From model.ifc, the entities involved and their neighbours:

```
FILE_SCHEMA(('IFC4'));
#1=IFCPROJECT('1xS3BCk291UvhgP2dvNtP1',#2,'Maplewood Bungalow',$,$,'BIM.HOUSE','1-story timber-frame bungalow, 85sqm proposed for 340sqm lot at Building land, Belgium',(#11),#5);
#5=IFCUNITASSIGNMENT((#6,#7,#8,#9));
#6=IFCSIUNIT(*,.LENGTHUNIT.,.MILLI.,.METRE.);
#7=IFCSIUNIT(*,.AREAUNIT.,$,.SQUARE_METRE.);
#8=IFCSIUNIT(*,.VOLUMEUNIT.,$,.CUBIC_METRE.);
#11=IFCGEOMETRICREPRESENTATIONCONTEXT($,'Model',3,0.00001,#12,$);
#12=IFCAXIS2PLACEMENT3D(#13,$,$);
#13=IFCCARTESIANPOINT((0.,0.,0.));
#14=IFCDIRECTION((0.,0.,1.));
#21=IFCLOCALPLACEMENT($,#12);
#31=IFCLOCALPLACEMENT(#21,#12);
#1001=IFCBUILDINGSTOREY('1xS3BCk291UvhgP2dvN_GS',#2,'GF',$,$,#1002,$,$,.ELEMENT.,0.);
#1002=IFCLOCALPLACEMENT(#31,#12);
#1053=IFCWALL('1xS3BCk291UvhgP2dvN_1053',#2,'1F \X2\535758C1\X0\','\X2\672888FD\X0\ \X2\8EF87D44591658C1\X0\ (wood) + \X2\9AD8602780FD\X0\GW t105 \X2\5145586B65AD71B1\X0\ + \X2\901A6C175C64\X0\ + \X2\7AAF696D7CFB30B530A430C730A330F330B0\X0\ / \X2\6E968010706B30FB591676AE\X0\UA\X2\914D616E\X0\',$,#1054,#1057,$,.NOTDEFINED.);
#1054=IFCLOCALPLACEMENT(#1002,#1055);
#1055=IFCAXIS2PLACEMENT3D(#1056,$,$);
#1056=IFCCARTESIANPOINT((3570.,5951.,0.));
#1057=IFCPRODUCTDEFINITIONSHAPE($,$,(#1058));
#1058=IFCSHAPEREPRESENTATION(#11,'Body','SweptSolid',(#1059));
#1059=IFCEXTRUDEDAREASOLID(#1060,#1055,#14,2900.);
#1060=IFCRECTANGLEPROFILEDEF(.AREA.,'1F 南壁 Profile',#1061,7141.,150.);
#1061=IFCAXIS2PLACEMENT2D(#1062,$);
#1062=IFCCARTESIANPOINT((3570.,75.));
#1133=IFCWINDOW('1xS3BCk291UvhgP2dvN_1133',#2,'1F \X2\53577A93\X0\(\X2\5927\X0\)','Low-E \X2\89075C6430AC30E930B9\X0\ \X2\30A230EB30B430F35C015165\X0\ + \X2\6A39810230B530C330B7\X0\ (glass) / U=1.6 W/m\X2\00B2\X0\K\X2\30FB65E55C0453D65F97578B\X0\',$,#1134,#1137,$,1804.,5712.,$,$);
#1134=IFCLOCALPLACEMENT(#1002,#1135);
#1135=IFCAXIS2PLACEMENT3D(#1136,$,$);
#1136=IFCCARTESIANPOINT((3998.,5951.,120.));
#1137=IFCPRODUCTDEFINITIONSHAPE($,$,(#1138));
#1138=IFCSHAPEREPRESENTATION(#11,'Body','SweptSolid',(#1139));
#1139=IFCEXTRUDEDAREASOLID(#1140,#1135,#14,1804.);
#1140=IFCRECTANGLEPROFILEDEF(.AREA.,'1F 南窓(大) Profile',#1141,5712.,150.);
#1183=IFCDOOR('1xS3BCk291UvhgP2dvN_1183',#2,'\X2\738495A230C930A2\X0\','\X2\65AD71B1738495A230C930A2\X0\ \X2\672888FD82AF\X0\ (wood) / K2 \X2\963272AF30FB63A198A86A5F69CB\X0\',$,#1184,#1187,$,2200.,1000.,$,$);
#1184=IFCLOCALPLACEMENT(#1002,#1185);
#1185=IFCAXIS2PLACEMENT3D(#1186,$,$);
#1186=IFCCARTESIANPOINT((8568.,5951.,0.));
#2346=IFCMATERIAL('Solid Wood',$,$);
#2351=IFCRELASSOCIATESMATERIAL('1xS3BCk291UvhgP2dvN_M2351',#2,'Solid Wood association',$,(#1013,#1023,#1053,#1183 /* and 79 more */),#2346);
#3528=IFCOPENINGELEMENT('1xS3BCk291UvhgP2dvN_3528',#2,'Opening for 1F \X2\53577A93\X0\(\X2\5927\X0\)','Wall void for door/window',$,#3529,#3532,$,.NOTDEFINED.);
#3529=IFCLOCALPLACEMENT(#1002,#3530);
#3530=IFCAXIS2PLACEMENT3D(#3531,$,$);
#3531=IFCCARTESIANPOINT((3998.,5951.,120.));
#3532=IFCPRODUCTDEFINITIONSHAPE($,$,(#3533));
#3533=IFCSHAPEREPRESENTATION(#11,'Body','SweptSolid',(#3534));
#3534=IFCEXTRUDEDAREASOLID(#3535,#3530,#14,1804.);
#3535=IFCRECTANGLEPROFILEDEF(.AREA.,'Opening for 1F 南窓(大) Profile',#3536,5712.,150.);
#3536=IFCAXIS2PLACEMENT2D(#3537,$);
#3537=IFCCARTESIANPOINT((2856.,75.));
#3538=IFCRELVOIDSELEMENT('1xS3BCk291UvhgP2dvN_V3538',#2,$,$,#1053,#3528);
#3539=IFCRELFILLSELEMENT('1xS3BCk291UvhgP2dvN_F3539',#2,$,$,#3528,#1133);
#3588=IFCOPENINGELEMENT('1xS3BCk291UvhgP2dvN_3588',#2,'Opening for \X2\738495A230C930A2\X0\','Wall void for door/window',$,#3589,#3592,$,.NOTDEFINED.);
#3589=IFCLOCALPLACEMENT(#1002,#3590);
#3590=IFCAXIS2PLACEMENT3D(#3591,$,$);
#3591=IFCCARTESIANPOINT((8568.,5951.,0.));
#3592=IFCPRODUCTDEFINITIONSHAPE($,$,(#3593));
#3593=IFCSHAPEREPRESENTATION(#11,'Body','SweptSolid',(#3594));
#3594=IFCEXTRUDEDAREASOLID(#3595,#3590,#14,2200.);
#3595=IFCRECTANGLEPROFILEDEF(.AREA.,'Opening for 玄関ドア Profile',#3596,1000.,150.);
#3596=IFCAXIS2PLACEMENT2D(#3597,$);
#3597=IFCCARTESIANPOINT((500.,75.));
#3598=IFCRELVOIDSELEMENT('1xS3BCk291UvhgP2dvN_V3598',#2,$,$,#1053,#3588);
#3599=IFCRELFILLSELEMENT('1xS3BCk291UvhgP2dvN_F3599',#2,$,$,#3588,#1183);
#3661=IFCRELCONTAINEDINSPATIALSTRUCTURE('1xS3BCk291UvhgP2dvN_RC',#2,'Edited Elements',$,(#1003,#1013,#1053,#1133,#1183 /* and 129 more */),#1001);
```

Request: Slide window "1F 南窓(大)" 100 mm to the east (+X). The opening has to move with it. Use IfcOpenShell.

```python
import ifcopenshell
import ifcopenshell.api.geometry
import ifcopenshell.util.placement
import ifcopenshell.util.unit

model = ifcopenshell.open("model.ifc")
unit_scale = ifcopenshell.util.unit.calculate_unit_scale(model)

window = model.by_id(1133)
opening = window.FillsVoids[0].RelatingOpeningElement
wall = opening.VoidsElements[0].RelatingBuildingElement

wall_matrix = ifcopenshell.util.placement.get_local_placement(wall.ObjectPlacement)
shift = wall_matrix[:3, 0] * 0.1 / unit_scale
before = ifcopenshell.util.placement.get_local_placement(window.ObjectPlacement)[:3, 3].copy()

# The window is not placed relative to its opening, so move both.
for product in (opening, window):
    matrix = ifcopenshell.util.placement.get_local_placement(product.ObjectPlacement)
    matrix[:3, 3] += shift
    ifcopenshell.api.geometry.edit_object_placement(model, product=product, matrix=matrix, is_si=False)

after = ifcopenshell.util.placement.get_local_placement(window.ObjectPlacement)[:3, 3]
print("window moved by", (after - before).round(3) + 0.0)

model.write("model_rev.ifc")
```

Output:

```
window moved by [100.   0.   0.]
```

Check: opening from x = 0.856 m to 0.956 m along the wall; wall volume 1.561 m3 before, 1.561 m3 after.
